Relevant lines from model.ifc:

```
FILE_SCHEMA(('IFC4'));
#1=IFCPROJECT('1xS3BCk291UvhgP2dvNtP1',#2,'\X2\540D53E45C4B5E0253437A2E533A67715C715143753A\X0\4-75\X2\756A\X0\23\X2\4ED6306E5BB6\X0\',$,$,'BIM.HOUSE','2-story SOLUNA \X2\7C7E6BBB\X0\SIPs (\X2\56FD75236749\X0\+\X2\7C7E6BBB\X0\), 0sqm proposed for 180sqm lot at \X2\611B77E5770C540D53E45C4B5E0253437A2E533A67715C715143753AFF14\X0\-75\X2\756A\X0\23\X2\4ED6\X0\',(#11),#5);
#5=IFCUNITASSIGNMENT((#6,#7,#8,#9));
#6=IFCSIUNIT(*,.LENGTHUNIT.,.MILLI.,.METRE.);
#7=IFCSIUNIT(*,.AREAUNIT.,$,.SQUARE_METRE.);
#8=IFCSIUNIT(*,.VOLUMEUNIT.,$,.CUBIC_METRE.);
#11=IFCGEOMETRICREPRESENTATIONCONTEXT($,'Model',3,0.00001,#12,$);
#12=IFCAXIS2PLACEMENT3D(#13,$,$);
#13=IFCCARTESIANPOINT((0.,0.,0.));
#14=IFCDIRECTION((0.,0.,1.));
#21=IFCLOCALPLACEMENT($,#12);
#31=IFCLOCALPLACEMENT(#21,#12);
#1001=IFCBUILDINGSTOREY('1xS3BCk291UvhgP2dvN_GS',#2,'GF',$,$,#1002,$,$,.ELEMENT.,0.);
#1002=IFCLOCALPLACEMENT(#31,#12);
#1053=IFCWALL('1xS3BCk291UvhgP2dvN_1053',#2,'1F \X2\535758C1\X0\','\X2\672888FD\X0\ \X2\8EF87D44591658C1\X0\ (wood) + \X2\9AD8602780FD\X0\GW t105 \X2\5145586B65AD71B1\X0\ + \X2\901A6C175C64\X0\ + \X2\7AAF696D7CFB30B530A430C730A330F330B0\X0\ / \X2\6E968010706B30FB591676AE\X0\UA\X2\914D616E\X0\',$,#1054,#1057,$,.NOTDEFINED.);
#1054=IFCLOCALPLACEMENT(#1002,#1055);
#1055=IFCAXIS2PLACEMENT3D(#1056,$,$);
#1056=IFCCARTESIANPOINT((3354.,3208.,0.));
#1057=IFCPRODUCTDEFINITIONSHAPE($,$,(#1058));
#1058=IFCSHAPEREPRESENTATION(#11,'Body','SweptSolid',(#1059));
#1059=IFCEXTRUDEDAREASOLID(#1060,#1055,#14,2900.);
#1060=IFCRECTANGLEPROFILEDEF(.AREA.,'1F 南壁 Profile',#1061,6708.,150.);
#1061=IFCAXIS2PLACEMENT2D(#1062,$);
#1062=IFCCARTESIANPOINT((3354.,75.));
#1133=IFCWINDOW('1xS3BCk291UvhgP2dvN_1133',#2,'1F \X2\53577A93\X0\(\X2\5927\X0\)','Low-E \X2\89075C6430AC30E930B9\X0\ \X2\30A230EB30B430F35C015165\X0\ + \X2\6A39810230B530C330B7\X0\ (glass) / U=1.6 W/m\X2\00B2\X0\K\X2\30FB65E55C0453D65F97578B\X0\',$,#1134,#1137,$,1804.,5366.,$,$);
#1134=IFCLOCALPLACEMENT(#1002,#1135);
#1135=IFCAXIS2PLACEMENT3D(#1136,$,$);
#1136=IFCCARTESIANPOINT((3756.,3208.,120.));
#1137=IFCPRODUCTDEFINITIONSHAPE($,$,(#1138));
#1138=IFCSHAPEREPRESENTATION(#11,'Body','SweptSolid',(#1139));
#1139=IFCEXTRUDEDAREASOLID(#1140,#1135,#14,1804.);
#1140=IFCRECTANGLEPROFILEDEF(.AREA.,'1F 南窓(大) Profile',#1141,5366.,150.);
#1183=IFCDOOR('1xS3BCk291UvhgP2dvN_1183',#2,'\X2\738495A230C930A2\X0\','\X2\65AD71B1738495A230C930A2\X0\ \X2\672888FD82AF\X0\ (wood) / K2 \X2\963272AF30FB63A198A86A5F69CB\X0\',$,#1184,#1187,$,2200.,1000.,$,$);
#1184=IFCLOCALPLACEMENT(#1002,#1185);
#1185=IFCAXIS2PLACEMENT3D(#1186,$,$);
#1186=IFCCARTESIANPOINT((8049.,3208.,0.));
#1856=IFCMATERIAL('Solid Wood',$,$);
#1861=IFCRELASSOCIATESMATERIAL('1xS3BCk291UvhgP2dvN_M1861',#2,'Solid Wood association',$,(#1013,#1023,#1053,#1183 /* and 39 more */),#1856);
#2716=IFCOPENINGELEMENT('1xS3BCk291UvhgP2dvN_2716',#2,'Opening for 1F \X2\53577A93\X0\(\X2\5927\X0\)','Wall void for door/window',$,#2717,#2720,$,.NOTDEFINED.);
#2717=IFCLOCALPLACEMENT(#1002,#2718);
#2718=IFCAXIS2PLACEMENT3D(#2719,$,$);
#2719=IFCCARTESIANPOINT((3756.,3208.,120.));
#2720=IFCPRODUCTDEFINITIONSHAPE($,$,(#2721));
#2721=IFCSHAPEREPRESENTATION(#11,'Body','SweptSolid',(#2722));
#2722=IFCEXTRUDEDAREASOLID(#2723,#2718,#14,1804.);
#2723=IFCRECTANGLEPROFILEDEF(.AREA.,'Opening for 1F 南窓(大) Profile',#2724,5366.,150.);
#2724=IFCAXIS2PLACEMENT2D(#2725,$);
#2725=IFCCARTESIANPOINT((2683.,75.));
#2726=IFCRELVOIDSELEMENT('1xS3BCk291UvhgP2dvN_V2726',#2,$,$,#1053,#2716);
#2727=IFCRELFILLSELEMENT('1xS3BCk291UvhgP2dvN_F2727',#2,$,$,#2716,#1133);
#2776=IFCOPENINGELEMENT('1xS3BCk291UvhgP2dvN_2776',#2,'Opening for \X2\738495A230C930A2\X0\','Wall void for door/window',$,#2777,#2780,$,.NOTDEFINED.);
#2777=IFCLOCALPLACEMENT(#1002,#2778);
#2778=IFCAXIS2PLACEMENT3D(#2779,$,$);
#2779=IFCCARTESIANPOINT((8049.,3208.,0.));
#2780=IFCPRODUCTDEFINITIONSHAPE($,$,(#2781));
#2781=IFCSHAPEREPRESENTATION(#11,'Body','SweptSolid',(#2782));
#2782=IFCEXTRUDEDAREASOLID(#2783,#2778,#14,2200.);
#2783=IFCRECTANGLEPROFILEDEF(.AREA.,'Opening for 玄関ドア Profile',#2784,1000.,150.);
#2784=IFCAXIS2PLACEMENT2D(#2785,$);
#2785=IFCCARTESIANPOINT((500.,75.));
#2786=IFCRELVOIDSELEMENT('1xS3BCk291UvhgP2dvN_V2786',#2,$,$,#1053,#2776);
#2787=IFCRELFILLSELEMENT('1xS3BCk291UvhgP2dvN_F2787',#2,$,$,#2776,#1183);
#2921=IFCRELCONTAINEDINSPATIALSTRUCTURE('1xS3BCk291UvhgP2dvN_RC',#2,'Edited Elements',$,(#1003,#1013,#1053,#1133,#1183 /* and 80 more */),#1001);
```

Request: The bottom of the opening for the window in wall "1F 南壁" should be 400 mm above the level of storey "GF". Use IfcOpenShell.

```python
import numpy as np
import ifcopenshell
import ifcopenshell.api.geometry
import ifcopenshell.geom
import ifcopenshell.util.element
import ifcopenshell.util.placement
import ifcopenshell.util.shape
import ifcopenshell.util.unit

model = ifcopenshell.open("model.ifc")
unit_scale = ifcopenshell.util.unit.calculate_unit_scale(model)

window = model.by_guid("1xS3BCk291UvhgP2dvN_1133")
opening = window.FillsVoids[0].RelatingOpeningElement
storey = ifcopenshell.util.element.get_container(window, ifc_class="IfcBuildingStorey")
level = ifcopenshell.util.placement.get_local_placement(storey.ObjectPlacement)[2, 3]

# The opening's origin need not be at the sill, so measure its lowest point.
shape = ifcopenshell.geom.create_shape(ifcopenshell.geom.settings(), opening)
bottom = ifcopenshell.util.shape.get_shape_bottom_elevation(shape, shape.geometry) / unit_scale
dz = level + 0.4 / unit_scale - bottom

shift = np.array([0.0, 0.0, dz])
# The window is not placed relative to its opening, so move both.
for product in (opening, window):
    matrix = ifcopenshell.util.placement.get_local_placement(product.ObjectPlacement)
    matrix[:3, 3] += shift
    ifcopenshell.api.geometry.edit_object_placement(model, product=product, matrix=matrix, is_si=False)

print(f"moved by {dz * unit_scale:+.3f} m")

model.write("model_edited.ifc")
```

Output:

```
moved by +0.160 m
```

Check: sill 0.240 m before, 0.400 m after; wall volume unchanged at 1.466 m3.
